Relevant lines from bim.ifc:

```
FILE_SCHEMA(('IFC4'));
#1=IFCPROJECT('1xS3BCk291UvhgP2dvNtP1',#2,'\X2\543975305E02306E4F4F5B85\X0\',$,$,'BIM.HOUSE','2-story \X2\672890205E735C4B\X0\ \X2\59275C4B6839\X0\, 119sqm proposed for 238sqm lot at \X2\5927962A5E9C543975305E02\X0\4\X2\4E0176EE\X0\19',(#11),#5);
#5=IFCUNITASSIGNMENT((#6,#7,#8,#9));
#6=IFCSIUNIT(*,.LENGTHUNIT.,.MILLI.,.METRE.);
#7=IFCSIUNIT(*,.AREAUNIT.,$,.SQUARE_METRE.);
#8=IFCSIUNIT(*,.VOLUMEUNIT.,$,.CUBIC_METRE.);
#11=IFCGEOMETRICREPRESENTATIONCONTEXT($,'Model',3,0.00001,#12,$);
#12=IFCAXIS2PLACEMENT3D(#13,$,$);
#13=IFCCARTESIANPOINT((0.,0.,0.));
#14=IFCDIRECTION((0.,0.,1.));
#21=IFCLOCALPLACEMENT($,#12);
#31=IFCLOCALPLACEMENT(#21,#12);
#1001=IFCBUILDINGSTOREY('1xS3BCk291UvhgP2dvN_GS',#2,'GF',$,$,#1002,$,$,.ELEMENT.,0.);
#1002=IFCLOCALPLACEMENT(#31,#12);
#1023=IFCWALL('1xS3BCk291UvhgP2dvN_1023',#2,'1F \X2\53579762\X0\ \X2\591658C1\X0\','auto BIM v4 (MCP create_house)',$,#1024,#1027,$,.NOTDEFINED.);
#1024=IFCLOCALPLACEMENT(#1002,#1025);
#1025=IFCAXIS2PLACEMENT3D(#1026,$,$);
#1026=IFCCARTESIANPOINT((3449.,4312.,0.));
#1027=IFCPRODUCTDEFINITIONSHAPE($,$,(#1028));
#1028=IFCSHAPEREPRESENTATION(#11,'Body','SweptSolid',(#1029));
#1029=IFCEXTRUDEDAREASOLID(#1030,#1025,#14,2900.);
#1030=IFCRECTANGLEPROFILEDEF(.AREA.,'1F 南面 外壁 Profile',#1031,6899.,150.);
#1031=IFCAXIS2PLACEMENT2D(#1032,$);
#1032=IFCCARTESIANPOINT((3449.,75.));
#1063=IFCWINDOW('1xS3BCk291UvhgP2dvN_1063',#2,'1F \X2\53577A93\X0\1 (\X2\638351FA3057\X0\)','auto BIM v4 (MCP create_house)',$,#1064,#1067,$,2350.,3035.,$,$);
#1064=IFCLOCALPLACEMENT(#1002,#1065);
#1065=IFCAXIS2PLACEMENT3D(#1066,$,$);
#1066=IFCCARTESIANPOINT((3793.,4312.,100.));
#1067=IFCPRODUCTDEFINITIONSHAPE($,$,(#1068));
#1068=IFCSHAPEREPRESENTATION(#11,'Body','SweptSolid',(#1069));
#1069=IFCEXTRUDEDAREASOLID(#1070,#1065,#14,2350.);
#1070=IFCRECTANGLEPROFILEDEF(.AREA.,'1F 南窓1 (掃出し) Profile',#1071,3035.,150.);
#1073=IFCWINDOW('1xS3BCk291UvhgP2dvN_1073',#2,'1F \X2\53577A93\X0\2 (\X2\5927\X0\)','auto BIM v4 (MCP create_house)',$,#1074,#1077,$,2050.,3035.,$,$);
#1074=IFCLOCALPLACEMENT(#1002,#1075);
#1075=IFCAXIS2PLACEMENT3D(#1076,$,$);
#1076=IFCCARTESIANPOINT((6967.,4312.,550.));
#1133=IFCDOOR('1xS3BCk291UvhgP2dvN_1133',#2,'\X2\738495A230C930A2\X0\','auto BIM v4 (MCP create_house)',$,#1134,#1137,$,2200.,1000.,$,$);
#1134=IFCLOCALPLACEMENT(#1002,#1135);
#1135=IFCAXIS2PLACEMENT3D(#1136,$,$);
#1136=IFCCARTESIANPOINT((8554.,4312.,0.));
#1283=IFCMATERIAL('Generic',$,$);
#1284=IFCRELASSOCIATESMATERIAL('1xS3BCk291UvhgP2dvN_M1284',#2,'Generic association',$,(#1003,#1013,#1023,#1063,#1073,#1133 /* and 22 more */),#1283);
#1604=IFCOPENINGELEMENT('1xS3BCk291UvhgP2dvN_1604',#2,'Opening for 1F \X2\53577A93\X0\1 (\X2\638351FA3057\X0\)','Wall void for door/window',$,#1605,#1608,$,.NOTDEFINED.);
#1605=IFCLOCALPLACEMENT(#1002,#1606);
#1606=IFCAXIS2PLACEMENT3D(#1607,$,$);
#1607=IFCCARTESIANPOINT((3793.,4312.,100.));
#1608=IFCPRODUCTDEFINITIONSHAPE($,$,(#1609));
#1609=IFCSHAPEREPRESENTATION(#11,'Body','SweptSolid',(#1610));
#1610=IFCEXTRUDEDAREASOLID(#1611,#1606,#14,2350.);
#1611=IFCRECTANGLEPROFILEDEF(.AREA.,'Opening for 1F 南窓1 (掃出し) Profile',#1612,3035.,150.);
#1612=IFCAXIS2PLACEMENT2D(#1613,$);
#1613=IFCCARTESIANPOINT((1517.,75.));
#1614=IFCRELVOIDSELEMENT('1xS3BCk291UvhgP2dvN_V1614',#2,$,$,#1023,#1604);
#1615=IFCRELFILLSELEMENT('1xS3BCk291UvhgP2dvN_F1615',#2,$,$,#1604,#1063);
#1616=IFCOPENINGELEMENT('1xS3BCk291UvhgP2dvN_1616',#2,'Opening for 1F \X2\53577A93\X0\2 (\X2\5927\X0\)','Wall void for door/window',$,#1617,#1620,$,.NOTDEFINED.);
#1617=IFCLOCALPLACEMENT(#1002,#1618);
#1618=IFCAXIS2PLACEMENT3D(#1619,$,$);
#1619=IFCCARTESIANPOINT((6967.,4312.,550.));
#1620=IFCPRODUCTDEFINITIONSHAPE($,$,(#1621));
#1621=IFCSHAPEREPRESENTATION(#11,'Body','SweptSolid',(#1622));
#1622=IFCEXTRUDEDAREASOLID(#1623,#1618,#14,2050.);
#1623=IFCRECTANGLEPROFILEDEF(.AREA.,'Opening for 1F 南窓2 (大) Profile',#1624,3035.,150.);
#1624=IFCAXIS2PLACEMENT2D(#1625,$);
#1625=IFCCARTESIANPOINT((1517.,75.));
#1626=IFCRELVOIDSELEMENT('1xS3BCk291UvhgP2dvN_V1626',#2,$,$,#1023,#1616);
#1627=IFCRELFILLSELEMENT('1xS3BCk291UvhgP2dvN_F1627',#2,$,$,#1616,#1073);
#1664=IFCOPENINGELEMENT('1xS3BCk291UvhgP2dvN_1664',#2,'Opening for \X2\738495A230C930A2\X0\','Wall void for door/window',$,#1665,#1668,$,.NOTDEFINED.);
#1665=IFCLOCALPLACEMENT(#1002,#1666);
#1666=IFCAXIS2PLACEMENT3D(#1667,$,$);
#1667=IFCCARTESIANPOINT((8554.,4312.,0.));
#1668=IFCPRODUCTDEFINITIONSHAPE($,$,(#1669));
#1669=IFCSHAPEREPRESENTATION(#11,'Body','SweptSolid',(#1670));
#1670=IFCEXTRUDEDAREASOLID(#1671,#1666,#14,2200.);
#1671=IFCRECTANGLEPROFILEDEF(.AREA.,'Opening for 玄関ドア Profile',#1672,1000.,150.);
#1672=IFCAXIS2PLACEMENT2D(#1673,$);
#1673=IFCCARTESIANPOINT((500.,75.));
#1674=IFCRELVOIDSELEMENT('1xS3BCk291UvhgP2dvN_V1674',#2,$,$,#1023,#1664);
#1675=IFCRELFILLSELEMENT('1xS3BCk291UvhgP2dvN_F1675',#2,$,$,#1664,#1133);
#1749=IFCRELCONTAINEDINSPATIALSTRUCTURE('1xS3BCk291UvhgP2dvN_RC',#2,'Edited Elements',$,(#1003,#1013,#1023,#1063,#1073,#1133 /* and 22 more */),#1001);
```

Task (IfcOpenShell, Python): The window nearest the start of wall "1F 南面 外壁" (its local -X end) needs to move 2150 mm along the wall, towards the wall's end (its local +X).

```python
import ifcopenshell
import ifcopenshell.api.geometry
import ifcopenshell.util.placement

model = ifcopenshell.open("bim.ifc")

window = model.by_id(1063)
opening = window.FillsVoids[0].RelatingOpeningElement
wall = opening.VoidsElements[0].RelatingBuildingElement

wall_matrix = ifcopenshell.util.placement.get_local_placement(wall.ObjectPlacement)
shift = wall_matrix[:3, 0] * 2150.0
before = ifcopenshell.util.placement.get_local_placement(window.ObjectPlacement)[:3, 3].copy()

# The window is not placed relative to its opening, so move both.
for product in (opening, window):
    matrix = ifcopenshell.util.placement.get_local_placement(product.ObjectPlacement)
    matrix[:3, 3] += shift
    ifcopenshell.api.geometry.edit_object_placement(model, product=product, matrix=matrix, is_si=False)

after = ifcopenshell.util.placement.get_local_placement(window.ObjectPlacement)[:3, 3]
print("window moved by", (after - before).round(3) + 0.0)

model.write("bim_v2.ifc")
```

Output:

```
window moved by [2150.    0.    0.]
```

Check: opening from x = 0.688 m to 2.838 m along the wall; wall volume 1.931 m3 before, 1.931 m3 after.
